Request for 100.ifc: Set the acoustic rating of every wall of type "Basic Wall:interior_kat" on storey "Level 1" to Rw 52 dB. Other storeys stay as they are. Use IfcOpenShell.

First a look at what the model holds.

```python
import ifcopenshell
import ifcopenshell.util.element

model = ifcopenshell.open("100.ifc")
print(model.schema)
storey = next(s for s in model.by_type("IfcBuildingStorey") if s.Name == "Level 1")
walls = [e for e in ifcopenshell.util.element.get_decomposition(storey) if e.is_a("IfcWall")]
seen = {}
for e in walls:
    element_type = ifcopenshell.util.element.get_type(e)
    key = (element_type.Name if element_type != e and element_type else None, ifcopenshell.util.element.get_pset(e, "Pset_WallCommon", "AcousticRating"))
    seen[key] = seen.get(key, 0) + 1
for (name, value), count in sorted(seen.items(), key=str):
    print(count, "x", name, "|", value)
```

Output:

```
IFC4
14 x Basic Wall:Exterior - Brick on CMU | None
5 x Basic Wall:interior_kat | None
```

```python
import ifcopenshell
import ifcopenshell.api.pset
import ifcopenshell.util.element

model = ifcopenshell.open("100.ifc")

storey = next(s for s in model.by_type("IfcBuildingStorey") if s.Name == "Level 1")
walls = [e for e in ifcopenshell.util.element.get_decomposition(storey) if e.is_a("IfcWall")]

count = 0
for e in walls:
    element_type = ifcopenshell.util.element.get_type(e)
    if element_type in (None, e) or element_type.Name != "Basic Wall:interior_kat":
        continue
    # add_pset returns the element's existing set when there is one.
    pset = ifcopenshell.api.pset.add_pset(model, product=e, name="Pset_WallCommon")
    ifcopenshell.api.pset.edit_pset(model, pset=pset, properties={"AcousticRating": "Rw 52 dB"})
    count += 1

print(count, "walls updated")

model.write("100_updated.ifc")
```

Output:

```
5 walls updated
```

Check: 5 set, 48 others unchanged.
